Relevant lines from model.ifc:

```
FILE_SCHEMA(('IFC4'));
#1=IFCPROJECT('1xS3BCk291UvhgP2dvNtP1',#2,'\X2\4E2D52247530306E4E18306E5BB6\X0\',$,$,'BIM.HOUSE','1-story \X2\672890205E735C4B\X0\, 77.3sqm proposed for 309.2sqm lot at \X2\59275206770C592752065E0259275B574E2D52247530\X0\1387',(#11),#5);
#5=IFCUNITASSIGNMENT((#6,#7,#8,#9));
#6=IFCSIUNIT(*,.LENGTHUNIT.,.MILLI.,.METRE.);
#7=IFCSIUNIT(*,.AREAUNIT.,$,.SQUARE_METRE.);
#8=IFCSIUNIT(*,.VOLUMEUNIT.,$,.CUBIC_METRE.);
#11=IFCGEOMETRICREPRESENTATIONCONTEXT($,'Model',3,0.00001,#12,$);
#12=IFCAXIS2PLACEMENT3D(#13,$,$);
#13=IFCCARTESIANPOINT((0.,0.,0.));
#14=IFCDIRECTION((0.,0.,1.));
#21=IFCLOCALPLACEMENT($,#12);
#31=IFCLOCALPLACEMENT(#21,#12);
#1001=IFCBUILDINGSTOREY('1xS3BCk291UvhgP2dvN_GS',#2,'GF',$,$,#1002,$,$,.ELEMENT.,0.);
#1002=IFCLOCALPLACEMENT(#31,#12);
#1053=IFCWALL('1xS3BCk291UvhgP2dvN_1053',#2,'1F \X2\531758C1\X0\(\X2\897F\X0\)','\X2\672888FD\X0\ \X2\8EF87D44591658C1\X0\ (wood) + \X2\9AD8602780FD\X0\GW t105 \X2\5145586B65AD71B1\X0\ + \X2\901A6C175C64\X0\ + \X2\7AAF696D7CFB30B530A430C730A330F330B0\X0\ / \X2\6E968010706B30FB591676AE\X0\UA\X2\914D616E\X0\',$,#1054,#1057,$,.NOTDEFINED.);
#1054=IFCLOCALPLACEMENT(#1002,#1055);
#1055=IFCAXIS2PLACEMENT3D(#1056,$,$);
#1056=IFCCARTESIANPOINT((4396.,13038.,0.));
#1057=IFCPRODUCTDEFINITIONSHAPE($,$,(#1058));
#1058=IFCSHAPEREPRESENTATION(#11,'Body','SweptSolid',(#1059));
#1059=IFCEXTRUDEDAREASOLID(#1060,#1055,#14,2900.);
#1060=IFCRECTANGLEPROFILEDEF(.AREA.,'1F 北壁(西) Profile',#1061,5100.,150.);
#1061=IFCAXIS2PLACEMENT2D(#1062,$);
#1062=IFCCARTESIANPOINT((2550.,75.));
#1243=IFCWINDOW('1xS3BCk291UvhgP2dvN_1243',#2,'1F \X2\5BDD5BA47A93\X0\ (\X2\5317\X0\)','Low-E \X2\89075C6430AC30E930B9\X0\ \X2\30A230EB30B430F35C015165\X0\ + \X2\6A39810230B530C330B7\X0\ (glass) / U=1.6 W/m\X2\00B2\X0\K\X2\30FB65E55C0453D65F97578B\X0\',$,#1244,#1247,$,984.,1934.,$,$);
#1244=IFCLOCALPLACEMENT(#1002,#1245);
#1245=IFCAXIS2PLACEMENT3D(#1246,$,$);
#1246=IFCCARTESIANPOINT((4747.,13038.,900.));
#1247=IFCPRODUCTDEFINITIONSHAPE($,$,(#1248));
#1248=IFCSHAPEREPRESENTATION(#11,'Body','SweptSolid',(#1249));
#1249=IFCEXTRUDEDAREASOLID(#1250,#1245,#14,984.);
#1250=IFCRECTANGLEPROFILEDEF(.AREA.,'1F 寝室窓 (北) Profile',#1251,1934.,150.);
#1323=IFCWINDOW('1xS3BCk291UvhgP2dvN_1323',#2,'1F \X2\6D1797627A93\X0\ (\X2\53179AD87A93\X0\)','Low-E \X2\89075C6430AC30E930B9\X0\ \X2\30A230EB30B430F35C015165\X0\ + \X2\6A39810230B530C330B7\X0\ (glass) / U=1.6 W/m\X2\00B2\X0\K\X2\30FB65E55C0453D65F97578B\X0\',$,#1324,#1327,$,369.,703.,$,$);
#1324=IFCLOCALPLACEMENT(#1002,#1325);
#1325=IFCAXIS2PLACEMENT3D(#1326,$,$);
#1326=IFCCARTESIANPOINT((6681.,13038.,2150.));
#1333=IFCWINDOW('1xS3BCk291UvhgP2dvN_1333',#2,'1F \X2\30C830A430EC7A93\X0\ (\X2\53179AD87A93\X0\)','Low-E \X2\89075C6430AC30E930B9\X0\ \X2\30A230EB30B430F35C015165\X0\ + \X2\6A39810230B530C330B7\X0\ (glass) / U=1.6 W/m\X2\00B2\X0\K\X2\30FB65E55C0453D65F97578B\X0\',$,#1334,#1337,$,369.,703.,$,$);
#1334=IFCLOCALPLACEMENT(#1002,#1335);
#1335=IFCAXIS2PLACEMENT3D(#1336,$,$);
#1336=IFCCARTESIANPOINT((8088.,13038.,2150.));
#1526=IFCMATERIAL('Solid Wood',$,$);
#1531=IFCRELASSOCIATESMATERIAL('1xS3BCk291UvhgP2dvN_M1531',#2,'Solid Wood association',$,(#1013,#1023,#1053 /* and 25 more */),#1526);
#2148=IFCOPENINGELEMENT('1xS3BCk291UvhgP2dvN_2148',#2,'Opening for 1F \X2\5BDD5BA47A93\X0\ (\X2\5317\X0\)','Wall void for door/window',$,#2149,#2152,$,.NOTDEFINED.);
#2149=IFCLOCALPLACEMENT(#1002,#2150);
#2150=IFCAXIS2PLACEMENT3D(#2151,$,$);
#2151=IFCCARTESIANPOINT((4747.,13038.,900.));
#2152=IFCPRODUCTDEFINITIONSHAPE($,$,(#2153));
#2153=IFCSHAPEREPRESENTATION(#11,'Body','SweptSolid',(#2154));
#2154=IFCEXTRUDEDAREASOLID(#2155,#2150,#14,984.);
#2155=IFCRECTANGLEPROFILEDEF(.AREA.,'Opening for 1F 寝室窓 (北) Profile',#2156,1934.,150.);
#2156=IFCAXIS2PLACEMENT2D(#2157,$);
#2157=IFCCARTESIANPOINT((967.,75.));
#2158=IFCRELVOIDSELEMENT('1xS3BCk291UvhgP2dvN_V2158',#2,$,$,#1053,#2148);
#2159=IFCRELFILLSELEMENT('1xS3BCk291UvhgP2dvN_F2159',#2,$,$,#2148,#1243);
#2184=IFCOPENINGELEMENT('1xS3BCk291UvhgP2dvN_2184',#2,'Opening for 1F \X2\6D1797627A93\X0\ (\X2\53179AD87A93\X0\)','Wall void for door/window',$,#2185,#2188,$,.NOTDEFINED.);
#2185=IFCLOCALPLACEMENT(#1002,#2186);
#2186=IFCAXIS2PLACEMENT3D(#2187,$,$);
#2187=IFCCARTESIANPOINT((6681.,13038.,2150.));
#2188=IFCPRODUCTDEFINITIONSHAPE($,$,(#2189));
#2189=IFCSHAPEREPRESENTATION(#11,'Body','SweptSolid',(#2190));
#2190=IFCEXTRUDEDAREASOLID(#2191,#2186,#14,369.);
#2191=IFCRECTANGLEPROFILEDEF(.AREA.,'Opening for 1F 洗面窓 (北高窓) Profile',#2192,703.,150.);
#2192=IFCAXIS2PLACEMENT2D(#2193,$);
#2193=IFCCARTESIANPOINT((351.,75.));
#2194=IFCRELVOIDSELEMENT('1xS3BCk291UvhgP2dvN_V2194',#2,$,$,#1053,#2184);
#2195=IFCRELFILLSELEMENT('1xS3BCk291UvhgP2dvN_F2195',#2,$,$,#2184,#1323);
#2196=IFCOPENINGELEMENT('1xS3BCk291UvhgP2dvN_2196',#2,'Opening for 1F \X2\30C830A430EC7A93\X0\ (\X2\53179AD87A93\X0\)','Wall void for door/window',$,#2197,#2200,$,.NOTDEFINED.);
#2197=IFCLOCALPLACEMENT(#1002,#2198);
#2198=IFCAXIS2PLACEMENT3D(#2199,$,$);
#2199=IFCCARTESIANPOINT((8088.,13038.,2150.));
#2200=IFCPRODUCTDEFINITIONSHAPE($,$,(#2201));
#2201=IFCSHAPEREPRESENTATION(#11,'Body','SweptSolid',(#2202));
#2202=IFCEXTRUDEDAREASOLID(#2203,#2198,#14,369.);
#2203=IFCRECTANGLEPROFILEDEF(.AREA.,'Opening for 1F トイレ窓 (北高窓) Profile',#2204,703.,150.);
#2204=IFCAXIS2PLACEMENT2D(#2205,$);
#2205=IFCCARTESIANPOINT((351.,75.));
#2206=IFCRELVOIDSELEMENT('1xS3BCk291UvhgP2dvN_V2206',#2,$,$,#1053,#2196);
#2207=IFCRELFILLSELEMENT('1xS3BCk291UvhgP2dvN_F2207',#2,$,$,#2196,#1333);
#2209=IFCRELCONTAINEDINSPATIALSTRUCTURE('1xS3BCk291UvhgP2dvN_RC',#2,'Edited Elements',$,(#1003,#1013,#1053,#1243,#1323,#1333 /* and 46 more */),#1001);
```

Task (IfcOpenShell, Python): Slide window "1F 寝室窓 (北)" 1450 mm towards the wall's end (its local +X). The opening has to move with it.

```python
import ifcopenshell
import ifcopenshell.api.geometry
import ifcopenshell.util.placement
import ifcopenshell.util.unit

model = ifcopenshell.open("model.ifc")
unit_scale = ifcopenshell.util.unit.calculate_unit_scale(model)

window = model.by_guid("1xS3BCk291UvhgP2dvN_1243")
opening = window.FillsVoids[0].RelatingOpeningElement
wall = opening.VoidsElements[0].RelatingBuildingElement

wall_matrix = ifcopenshell.util.placement.get_local_placement(wall.ObjectPlacement)
shift = wall_matrix[:3, 0] * 1.45 / unit_scale
before = ifcopenshell.util.placement.get_local_placement(window.ObjectPlacement)[:3, 3].copy()

# The window is not placed relative to its opening, so move both.
for product in (opening, window):
    matrix = ifcopenshell.util.placement.get_local_placement(product.ObjectPlacement)
    matrix[:3, 3] += shift
    ifcopenshell.api.geometry.edit_object_placement(model, product=product, matrix=matrix, is_si=False)

after = ifcopenshell.util.placement.get_local_placement(window.ObjectPlacement)[:3, 3]
print("window moved by", (after - before).round(3) + 0.0)

model.write("model_rev.ifc")
```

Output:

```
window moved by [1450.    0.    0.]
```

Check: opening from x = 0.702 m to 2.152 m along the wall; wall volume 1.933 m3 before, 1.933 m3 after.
